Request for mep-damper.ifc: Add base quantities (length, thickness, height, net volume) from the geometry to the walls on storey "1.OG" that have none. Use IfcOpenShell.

First a look at what the model holds.

```python
import ifcopenshell
import ifcopenshell.util.element
import ifcopenshell.util.unit

model = ifcopenshell.open("mep-damper.ifc")
print(model.schema)
for unit_type in ("LENGTHUNIT", "AREAUNIT", "VOLUMEUNIT"):
    print(unit_type, ifcopenshell.util.unit.calculate_unit_scale(model, unit_type))
storey = next(s for s in model.by_type("IfcBuildingStorey") if s.Name == "1.OG")
walls = [e for e in ifcopenshell.util.element.get_decomposition(storey) if e.is_a("IfcWall")]
for e in sorted(walls, key=lambda e: e.id()):
    print(e.id(), e.is_a(), e.Name, list(ifcopenshell.util.element.get_psets(e, qtos_only=True)), sep=" | ")
```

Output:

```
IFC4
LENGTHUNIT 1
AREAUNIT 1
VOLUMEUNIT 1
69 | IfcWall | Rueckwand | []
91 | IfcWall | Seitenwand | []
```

```python
import ifcopenshell
import ifcopenshell.api.pset
import ifcopenshell.geom
import ifcopenshell.util.element
import ifcopenshell.util.shape
import ifcopenshell.util.unit

model = ifcopenshell.open("mep-damper.ifc")
unit_scale = ifcopenshell.util.unit.calculate_unit_scale(model)
volume_scale = ifcopenshell.util.unit.calculate_unit_scale(model, "VOLUMEUNIT")
settings = ifcopenshell.geom.settings()

storey = next(s for s in model.by_type("IfcBuildingStorey") if s.Name == "1.OG")
walls = [e for e in ifcopenshell.util.element.get_decomposition(storey) if e.is_a("IfcWall")]

for e in sorted(walls, key=lambda e: e.id()):
    if ifcopenshell.util.element.get_psets(e, qtos_only=True, should_inherit=False):
        continue
    # Geometry comes back in metres, in the element's own axes.
    shape = ifcopenshell.geom.create_shape(settings, e)
    values = {
        "Length": ifcopenshell.util.shape.get_x(shape.geometry) / unit_scale,
        "Width": ifcopenshell.util.shape.get_y(shape.geometry) / unit_scale,
        "Height": ifcopenshell.util.shape.get_z(shape.geometry) / unit_scale,
        "NetVolume": ifcopenshell.util.shape.get_volume(shape.geometry) / volume_scale,
    }
    qto = ifcopenshell.api.pset.add_qto(model, product=e, name="Qto_WallBaseQuantities")
    ifcopenshell.api.pset.edit_qto(model, qto=qto, properties=values)
    print(e.id(), {k: round(v, 3) for k, v in values.items()})

model.write("mep-damper_v2.ifc")
```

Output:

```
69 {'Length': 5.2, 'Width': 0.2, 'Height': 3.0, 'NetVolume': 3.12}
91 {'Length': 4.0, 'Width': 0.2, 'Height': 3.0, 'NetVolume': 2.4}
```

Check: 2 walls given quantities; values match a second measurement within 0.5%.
